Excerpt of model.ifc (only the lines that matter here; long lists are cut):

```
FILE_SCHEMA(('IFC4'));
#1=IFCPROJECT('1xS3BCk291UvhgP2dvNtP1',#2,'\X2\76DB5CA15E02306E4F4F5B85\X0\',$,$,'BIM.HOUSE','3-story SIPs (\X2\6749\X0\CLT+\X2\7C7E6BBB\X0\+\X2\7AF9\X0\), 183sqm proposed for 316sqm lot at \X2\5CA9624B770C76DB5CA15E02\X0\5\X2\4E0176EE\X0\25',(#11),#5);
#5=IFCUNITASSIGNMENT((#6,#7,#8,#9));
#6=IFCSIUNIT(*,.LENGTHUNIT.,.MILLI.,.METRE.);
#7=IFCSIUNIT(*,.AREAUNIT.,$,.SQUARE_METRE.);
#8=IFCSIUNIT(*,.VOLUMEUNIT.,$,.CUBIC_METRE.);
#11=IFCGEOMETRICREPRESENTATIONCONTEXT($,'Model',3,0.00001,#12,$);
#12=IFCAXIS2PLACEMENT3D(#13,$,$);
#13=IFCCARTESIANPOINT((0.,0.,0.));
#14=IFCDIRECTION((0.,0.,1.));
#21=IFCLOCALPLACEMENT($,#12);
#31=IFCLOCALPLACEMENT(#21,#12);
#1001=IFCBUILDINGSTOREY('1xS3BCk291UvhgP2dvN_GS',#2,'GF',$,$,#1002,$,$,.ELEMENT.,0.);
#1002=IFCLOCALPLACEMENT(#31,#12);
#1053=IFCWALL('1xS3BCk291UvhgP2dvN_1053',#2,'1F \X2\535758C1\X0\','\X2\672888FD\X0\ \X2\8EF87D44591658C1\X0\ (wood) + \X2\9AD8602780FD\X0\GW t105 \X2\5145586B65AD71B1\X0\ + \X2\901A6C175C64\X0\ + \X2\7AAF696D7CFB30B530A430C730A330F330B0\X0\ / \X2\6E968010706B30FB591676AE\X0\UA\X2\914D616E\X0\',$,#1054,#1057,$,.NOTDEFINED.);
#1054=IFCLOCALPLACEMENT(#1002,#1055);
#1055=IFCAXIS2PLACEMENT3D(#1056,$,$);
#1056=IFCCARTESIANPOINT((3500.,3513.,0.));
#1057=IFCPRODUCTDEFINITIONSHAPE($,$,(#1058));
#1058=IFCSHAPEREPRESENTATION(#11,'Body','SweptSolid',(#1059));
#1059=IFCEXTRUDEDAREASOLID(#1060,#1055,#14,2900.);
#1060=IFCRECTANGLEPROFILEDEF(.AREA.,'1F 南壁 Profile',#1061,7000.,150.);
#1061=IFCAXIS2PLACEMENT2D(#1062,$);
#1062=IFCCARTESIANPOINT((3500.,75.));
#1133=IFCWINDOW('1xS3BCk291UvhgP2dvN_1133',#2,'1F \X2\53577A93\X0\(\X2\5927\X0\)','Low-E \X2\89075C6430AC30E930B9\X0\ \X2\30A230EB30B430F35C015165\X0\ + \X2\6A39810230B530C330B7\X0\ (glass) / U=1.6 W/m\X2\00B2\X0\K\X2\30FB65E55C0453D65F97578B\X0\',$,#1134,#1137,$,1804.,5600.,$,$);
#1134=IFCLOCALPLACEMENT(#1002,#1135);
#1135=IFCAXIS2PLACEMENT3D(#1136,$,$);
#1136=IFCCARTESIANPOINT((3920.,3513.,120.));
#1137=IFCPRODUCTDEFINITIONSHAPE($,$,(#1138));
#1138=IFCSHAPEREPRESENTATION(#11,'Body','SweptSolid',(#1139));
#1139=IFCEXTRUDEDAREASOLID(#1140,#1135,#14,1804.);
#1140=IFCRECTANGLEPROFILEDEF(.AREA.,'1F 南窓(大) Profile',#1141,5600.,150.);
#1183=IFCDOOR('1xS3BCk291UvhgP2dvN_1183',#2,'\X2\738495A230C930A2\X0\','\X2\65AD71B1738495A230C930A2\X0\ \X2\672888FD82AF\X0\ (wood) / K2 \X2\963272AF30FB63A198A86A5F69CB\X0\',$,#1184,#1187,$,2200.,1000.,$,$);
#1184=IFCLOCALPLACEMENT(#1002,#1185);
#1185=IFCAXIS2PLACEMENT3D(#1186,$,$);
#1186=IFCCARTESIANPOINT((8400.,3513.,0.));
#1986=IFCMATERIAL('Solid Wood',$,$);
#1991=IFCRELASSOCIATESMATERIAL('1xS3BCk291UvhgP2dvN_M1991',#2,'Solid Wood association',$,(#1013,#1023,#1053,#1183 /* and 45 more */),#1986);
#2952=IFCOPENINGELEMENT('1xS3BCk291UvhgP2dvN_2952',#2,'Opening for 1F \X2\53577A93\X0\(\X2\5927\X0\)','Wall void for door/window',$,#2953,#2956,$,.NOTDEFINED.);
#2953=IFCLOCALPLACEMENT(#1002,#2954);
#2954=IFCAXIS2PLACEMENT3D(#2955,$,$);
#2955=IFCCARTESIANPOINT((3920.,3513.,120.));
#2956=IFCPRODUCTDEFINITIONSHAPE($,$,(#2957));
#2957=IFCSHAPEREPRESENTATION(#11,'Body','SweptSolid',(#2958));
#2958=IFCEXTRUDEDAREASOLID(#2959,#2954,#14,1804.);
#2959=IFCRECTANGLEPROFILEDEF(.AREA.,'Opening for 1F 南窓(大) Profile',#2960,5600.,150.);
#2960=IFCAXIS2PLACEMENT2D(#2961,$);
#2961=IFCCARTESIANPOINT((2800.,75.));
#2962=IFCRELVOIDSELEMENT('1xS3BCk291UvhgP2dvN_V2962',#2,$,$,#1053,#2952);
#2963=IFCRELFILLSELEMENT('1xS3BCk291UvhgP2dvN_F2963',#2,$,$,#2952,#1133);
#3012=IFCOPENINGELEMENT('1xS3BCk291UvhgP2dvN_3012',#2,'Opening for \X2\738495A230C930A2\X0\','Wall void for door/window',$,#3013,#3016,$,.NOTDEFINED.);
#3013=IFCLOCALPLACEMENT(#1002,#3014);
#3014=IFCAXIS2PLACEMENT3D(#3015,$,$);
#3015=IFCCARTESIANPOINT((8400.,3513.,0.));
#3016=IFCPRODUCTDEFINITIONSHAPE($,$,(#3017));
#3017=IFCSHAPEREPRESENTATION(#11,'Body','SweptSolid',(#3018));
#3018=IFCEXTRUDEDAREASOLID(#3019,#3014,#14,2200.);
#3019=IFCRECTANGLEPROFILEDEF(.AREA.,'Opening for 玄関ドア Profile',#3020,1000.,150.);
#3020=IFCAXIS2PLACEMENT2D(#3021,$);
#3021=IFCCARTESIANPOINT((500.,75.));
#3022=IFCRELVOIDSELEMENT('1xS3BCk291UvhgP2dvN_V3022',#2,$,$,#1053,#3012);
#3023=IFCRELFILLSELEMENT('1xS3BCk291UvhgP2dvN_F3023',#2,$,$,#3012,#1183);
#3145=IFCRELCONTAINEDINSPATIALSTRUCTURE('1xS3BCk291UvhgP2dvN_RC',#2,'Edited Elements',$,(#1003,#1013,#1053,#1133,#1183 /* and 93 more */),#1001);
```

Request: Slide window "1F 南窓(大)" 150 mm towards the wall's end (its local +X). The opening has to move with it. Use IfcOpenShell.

```python
import ifcopenshell
import ifcopenshell.api.geometry
import ifcopenshell.util.placement
import ifcopenshell.util.unit

model = ifcopenshell.open("model.ifc")
unit_scale = ifcopenshell.util.unit.calculate_unit_scale(model)

window = model.by_guid("1xS3BCk291UvhgP2dvN_1133")
opening = window.FillsVoids[0].RelatingOpeningElement
wall = opening.VoidsElements[0].RelatingBuildingElement

wall_matrix = ifcopenshell.util.placement.get_local_placement(wall.ObjectPlacement)
shift = wall_matrix[:3, 0] * 0.15 / unit_scale
before = ifcopenshell.util.placement.get_local_placement(window.ObjectPlacement)[:3, 3].copy()

# The window is not placed relative to its opening, so move both.
for product in (opening, window):
    matrix = ifcopenshell.util.placement.get_local_placement(product.ObjectPlacement)
    matrix[:3, 3] += shift
    ifcopenshell.api.geometry.edit_object_placement(model, product=product, matrix=matrix, is_si=False)

after = ifcopenshell.util.placement.get_local_placement(window.ObjectPlacement)[:3, 3]
print("window moved by", (after - before).round(3) + 0.0)

model.write("model-out.ifc")
```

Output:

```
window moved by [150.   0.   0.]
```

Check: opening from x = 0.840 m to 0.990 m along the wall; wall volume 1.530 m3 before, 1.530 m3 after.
